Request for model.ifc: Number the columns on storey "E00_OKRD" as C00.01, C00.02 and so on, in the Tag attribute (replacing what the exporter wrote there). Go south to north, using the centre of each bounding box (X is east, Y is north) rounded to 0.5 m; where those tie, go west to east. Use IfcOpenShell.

First a look at what the model holds.

```python
import ifcopenshell
import ifcopenshell.util.element
import ifcopenshell.util.placement

model = ifcopenshell.open("model.ifc")
print(model.schema)
storey = next(s for s in model.by_type("IfcBuildingStorey") if s.Name == "E00_OKRD")
columns = [e for e in ifcopenshell.util.element.get_decomposition(storey) if e.is_a("IfcColumn")]
for e in sorted(columns, key=lambda e: e.id()):
    origin = ifcopenshell.util.placement.get_local_placement(e.ObjectPlacement)[:3, 3]
    print(e.id(), e.Tag, e.Name, origin.round(2) + 0.0, sep=" | ")
```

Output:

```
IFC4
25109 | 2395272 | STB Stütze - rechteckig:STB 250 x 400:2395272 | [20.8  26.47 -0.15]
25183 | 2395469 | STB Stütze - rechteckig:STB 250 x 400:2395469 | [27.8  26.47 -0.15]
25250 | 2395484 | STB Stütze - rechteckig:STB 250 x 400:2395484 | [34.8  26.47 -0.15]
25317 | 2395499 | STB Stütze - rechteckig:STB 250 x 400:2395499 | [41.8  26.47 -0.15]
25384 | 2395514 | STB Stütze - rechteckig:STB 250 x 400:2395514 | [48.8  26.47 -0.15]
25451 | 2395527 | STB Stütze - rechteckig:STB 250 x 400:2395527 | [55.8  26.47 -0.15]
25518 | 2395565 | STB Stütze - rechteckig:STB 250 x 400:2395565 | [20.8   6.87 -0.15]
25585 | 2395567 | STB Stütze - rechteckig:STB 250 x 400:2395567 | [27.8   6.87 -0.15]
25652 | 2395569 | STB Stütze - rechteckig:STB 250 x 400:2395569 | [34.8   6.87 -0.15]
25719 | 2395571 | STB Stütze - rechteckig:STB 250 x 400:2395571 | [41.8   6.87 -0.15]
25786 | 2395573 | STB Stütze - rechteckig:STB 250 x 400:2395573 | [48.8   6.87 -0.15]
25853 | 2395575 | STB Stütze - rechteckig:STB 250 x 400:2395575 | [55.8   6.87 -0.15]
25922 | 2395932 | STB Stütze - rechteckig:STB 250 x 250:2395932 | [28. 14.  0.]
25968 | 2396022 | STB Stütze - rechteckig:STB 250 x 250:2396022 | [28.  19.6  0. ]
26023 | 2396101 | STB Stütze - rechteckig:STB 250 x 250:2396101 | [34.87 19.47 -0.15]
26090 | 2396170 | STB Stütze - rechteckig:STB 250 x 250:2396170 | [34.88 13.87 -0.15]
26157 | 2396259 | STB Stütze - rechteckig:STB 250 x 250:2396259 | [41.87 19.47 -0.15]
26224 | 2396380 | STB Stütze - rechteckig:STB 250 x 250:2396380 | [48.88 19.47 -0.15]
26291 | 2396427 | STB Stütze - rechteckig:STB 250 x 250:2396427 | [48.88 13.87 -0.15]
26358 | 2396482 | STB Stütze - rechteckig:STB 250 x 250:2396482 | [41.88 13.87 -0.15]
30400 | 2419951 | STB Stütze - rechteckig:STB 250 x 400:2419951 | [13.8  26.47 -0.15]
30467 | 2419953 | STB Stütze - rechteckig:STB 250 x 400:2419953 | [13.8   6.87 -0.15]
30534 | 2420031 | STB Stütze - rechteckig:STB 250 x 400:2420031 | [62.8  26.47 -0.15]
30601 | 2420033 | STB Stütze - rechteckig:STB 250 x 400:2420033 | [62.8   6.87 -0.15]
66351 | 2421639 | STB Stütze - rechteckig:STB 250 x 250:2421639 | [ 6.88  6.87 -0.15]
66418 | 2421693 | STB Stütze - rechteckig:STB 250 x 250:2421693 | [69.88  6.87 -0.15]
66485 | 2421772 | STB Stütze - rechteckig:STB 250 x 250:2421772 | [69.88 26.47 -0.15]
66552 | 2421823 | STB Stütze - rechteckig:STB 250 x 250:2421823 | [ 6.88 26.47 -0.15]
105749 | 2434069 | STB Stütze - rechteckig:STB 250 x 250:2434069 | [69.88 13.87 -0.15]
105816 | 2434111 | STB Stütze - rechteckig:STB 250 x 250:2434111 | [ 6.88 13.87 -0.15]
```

```python
import ifcopenshell
import ifcopenshell.geom
import ifcopenshell.util.element
import ifcopenshell.util.shape

model = ifcopenshell.open("model.ifc")
settings = ifcopenshell.geom.settings()
settings.set("use-world-coords", True)


def centre(element):
    shape = ifcopenshell.geom.create_shape(settings, element)
    return ifcopenshell.util.shape.get_bbox_centroid(shape.geometry)


storey = next(s for s in model.by_type("IfcBuildingStorey") if s.Name == "E00_OKRD")
columns = [e for e in ifcopenshell.util.element.get_decomposition(storey) if e.is_a("IfcColumn")]

# Insertion points can sit at a corner or the storey origin, so sort by the geometry (in metres).
centres = {e: centre(e) for e in columns}
columns.sort(key=lambda e: (round(centres[e][1] / 0.5), centres[e][0]))

for i, e in enumerate(columns, start=1):
    number = f"C00.{i:02d}"
    e.Tag = number
    print(e.id(), number)

model.write("model_v2.ifc")
```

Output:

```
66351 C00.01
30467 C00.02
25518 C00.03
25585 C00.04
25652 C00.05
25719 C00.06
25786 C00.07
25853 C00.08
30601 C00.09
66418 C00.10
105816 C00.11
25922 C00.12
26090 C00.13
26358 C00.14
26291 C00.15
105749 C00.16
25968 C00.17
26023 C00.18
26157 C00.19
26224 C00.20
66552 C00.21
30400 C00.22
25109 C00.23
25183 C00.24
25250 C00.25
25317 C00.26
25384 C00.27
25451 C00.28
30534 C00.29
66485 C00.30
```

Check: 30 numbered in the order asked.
